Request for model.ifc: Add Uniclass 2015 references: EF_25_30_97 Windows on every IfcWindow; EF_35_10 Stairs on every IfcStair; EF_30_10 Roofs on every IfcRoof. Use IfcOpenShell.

First a look at what the model holds.

```python
import ifcopenshell

model = ifcopenshell.open("model.ifc")
print(model.schema)
print("classifications:", [c.Name for c in model.by_type("IfcClassification")])
for ifc_class in ("IfcDoor", "IfcRoof", "IfcStair", "IfcWall", "IfcWindow"):
    print(ifc_class, len(model.by_type(ifc_class)))
```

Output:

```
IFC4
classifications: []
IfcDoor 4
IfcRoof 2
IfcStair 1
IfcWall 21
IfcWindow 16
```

```python
import ifcopenshell
import ifcopenshell.api.classification

model = ifcopenshell.open("model.ifc")

system = ifcopenshell.api.classification.add_classification(model, classification="Uniclass 2015")

codes = {
    "IfcWindow": ("EF_25_30_97", "Windows"),
    "IfcStair": ("EF_35_10", "Stairs"),
    "IfcRoof": ("EF_30_10", "Roofs"),
}
for ifc_class, (code, name) in codes.items():
    products = model.by_type(ifc_class)
    ifcopenshell.api.classification.add_reference(
        model, products=products, classification=system, identification=code, name=name
    )
    print(code, len(products))

model.write("model-out.ifc")
```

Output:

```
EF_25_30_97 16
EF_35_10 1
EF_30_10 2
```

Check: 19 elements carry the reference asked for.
